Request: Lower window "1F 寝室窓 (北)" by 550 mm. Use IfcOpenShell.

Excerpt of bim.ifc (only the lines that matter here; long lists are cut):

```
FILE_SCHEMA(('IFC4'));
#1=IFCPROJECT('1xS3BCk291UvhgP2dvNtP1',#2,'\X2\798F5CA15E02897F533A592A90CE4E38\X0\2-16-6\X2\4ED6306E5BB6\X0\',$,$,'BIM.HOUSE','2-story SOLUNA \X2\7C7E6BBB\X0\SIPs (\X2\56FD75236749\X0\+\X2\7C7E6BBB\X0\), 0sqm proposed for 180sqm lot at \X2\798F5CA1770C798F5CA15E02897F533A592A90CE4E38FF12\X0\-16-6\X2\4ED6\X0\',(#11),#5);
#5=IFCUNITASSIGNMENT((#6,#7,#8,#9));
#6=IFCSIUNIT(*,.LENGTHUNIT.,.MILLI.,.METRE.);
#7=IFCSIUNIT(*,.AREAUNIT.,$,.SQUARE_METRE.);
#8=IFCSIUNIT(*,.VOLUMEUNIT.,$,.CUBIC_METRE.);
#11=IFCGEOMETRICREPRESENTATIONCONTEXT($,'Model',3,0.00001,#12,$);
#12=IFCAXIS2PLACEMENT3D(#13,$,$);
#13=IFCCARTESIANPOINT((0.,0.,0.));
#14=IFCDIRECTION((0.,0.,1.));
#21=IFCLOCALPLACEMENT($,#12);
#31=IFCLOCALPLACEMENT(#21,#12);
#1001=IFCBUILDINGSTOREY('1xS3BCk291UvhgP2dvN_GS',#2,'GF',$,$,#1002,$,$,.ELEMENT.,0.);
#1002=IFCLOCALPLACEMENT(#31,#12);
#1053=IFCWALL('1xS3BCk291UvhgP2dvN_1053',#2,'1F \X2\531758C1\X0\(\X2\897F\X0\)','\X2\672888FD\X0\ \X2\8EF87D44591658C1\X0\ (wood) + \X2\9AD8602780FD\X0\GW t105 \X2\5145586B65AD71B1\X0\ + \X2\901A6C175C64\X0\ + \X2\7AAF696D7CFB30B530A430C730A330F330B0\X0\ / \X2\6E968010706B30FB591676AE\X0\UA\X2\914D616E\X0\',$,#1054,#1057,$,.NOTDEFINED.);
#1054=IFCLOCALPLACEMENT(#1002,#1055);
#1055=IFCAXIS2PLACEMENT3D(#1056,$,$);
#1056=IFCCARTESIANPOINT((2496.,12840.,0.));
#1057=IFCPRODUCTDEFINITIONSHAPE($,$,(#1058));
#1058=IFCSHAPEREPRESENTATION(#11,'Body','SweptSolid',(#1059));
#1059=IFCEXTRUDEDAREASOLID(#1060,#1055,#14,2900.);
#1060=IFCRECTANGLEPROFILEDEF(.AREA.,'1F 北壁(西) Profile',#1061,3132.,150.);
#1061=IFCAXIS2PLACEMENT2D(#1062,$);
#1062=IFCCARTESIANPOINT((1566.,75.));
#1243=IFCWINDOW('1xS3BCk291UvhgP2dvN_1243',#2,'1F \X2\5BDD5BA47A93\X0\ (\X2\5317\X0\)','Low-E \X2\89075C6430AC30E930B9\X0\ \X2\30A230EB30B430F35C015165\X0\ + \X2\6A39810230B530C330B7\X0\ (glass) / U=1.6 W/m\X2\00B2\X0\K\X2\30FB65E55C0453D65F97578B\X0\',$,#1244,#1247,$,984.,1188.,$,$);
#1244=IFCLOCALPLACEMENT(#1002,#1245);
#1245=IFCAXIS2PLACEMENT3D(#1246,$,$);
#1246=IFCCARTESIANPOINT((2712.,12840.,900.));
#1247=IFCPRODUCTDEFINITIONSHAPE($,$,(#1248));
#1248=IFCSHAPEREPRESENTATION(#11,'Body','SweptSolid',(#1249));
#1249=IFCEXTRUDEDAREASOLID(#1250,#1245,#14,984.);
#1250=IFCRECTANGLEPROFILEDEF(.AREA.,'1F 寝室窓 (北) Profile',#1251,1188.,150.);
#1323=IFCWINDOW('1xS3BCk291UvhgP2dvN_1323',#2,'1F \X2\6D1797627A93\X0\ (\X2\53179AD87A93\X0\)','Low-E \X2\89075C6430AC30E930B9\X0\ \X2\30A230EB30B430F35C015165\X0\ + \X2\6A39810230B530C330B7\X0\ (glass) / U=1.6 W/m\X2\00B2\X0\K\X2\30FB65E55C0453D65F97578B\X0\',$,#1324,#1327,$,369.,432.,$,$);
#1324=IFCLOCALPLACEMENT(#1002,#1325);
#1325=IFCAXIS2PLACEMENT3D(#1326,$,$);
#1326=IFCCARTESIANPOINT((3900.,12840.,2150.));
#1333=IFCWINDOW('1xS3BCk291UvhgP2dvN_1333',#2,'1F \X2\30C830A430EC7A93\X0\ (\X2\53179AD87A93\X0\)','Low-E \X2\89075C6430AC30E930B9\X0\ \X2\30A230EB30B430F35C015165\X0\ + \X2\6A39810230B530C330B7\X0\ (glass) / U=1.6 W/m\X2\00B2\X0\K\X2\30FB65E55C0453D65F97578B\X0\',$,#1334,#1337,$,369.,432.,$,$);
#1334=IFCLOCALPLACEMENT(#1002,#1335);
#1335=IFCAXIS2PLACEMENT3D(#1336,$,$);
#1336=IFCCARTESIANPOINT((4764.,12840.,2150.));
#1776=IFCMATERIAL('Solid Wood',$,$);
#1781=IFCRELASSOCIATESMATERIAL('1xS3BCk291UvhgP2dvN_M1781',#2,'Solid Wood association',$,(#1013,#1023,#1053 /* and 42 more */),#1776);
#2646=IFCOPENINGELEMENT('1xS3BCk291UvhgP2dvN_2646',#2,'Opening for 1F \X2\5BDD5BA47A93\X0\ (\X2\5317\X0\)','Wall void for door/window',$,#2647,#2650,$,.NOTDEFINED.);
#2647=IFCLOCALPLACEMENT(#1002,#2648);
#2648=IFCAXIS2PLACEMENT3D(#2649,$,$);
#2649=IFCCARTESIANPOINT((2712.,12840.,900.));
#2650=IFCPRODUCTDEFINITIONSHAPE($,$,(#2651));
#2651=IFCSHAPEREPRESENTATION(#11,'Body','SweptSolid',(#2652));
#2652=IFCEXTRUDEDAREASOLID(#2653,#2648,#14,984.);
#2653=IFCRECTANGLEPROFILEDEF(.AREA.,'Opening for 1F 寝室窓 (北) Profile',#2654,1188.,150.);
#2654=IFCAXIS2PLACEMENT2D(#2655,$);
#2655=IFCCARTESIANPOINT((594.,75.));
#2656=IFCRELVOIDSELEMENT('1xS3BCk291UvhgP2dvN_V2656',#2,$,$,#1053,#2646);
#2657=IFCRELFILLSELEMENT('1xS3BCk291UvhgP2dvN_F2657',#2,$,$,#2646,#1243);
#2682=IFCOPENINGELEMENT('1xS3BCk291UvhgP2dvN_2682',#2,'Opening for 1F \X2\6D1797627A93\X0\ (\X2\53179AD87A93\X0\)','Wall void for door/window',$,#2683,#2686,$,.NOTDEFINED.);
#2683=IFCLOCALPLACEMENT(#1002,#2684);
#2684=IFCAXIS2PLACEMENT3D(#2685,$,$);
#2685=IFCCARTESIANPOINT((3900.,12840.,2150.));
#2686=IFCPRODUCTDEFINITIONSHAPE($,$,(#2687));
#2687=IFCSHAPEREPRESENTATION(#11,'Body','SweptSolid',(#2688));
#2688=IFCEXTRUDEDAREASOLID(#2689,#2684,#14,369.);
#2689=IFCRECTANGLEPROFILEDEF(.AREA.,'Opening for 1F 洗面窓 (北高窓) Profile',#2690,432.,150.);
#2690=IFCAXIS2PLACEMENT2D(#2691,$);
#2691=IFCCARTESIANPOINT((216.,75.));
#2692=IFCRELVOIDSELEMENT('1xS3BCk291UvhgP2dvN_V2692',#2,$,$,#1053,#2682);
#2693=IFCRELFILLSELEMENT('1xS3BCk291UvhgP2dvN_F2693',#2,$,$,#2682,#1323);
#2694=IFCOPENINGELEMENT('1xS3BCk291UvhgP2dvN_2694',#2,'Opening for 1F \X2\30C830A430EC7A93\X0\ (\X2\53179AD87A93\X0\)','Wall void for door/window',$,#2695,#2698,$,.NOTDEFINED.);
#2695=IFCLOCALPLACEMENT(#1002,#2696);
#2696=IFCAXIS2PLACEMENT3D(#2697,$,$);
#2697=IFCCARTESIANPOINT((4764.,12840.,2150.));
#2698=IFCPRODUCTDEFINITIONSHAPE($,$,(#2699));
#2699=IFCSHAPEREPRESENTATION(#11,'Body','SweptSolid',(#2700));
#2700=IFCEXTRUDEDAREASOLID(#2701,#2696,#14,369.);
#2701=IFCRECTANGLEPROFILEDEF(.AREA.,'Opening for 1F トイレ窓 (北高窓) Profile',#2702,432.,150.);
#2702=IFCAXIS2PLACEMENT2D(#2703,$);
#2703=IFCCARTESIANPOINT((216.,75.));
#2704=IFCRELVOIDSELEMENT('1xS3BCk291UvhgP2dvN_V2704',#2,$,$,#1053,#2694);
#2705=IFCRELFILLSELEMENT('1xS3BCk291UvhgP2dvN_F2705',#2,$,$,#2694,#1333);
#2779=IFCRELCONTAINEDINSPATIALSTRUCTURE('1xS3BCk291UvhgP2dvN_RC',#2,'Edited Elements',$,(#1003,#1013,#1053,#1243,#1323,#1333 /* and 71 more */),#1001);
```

```python
import numpy as np
import ifcopenshell
import ifcopenshell.api.geometry
import ifcopenshell.util.placement
import ifcopenshell.util.unit

model = ifcopenshell.open("bim.ifc")
unit_scale = ifcopenshell.util.unit.calculate_unit_scale(model)

window = model.by_guid("1xS3BCk291UvhgP2dvN_1243")
opening = window.FillsVoids[0].RelatingOpeningElement
dz = -550.0

shift = np.array([0.0, 0.0, dz])
# The window is not placed relative to its opening, so move both.
for product in (opening, window):
    matrix = ifcopenshell.util.placement.get_local_placement(product.ObjectPlacement)
    matrix[:3, 3] += shift
    ifcopenshell.api.geometry.edit_object_placement(model, product=product, matrix=matrix, is_si=False)

print(f"moved by {dz * unit_scale:+.3f} m")

model.write("bim_rev.ifc")
```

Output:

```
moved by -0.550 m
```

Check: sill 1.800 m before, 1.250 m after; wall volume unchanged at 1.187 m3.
